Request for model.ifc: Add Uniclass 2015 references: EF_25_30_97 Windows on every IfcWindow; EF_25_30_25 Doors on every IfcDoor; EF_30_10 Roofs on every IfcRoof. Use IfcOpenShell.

First a look at what the model holds.

```python
import ifcopenshell

model = ifcopenshell.open("model.ifc")
print(model.schema)
print("classifications:", [c.Name for c in model.by_type("IfcClassification")])
for ifc_class in ("IfcDoor", "IfcRoof", "IfcStair", "IfcWall", "IfcWindow"):
    print(ifc_class, len(model.by_type(ifc_class)))
```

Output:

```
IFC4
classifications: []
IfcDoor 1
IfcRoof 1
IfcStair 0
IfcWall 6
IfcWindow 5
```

```python
import ifcopenshell
import ifcopenshell.api.classification

model = ifcopenshell.open("model.ifc")

system = ifcopenshell.api.classification.add_classification(model, classification="Uniclass 2015")

codes = {
    "IfcWindow": ("EF_25_30_97", "Windows"),
    "IfcDoor": ("EF_25_30_25", "Doors"),
    "IfcRoof": ("EF_30_10", "Roofs"),
}
for ifc_class, (code, name) in codes.items():
    products = model.by_type(ifc_class)
    ifcopenshell.api.classification.add_reference(
        model, products=products, classification=system, identification=code, name=name
    )
    print(code, len(products))

model.write("model_v2.ifc")
```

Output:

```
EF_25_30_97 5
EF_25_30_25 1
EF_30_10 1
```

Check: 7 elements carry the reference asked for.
